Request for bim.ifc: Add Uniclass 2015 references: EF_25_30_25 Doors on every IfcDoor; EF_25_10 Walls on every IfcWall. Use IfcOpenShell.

First a look at what the model holds.

```python
import ifcopenshell

model = ifcopenshell.open("bim.ifc")
print(model.schema)
print("classifications:", [c.Name for c in model.by_type("IfcClassification")])
for ifc_class in ("IfcDoor", "IfcRoof", "IfcStair", "IfcWall", "IfcWindow"):
    print(ifc_class, len(model.by_type(ifc_class)))
```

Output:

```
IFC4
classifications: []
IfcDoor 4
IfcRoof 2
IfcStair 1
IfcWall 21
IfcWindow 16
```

```python
import ifcopenshell
import ifcopenshell.api.classification

model = ifcopenshell.open("bim.ifc")

system = ifcopenshell.api.classification.add_classification(model, classification="Uniclass 2015")

codes = {
    "IfcDoor": ("EF_25_30_25", "Doors"),
    "IfcWall": ("EF_25_10", "Walls"),
}
for ifc_class, (code, name) in codes.items():
    products = model.by_type(ifc_class)
    ifcopenshell.api.classification.add_reference(
        model, products=products, classification=system, identification=code, name=name
    )
    print(code, len(products))

model.write("bim_rev.ifc")
```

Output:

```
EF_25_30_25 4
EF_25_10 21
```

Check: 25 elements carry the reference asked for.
